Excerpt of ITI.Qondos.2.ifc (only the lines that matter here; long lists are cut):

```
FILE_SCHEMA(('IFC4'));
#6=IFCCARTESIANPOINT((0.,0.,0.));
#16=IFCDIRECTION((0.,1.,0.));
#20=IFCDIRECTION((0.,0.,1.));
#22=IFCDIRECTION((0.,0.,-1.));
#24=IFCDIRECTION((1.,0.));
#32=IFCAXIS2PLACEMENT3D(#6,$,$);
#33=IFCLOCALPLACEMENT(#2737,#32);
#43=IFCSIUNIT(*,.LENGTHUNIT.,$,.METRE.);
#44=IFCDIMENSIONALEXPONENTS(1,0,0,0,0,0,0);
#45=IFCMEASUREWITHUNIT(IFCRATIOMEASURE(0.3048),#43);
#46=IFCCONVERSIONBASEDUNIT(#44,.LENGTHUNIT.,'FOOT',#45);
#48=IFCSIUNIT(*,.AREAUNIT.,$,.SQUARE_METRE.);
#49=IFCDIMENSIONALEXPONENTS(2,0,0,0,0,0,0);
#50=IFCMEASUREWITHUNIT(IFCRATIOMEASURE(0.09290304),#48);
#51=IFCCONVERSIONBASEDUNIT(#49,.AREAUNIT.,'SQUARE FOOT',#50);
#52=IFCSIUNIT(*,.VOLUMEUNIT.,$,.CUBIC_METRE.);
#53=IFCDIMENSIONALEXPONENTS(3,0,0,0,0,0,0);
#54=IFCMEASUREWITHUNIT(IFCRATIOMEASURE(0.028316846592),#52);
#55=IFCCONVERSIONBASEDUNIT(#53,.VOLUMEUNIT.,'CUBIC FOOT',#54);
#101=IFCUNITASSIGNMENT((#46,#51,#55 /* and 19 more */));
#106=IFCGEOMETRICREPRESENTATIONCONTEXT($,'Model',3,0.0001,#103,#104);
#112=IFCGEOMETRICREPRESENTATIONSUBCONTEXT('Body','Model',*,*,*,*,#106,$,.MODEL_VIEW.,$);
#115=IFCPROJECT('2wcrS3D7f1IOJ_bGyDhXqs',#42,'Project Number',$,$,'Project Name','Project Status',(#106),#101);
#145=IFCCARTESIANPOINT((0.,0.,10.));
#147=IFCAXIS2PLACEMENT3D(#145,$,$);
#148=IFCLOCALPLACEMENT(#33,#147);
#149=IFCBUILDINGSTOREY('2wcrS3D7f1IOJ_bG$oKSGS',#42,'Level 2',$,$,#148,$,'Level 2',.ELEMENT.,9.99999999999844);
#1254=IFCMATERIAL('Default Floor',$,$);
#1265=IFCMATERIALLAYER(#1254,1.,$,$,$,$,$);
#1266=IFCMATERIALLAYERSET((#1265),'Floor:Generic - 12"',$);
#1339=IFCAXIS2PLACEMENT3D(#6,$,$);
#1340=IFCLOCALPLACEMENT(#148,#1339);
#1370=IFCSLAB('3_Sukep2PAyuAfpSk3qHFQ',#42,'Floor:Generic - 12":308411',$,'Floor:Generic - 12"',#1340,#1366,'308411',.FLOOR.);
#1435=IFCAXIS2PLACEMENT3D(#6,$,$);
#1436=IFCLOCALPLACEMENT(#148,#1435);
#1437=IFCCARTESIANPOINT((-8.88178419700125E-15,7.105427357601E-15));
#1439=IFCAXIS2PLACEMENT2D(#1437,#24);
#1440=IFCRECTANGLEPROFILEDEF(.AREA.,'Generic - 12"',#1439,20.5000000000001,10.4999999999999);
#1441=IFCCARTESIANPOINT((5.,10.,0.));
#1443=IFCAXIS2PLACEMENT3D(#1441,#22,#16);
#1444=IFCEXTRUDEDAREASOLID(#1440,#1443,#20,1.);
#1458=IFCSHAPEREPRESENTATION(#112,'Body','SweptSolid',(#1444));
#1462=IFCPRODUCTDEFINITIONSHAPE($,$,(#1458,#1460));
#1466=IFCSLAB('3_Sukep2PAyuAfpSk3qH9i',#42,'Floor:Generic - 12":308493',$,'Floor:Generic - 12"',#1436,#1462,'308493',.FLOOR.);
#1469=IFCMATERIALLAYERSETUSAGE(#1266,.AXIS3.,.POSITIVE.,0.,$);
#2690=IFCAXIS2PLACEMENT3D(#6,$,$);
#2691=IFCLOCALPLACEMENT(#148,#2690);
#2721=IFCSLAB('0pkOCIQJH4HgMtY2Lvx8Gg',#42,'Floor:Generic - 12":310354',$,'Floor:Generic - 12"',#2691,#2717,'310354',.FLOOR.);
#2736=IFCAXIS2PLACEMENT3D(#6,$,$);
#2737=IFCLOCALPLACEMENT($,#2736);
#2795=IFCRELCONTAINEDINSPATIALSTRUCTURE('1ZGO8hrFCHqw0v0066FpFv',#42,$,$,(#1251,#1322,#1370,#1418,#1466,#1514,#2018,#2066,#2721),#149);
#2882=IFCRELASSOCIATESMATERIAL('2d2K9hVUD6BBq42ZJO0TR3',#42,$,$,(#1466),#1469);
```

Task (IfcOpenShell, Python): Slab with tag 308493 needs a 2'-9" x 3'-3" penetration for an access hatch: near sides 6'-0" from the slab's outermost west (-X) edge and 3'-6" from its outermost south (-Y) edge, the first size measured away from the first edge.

```python
import numpy as np
import ifcopenshell
import ifcopenshell.api.feature
import ifcopenshell.api.geometry
import ifcopenshell.api.root
import ifcopenshell.geom
import ifcopenshell.util.placement
import ifcopenshell.util.representation
import ifcopenshell.util.shape
import ifcopenshell.util.unit

model = ifcopenshell.open("ITI.Qondos.2.ifc")
unit_scale = ifcopenshell.util.unit.calculate_unit_scale(model)
settings = ifcopenshell.geom.settings()


def volume(element):
    """Net volume in cubic metres, openings subtracted."""
    shape = ifcopenshell.geom.create_shape(settings, element)
    return ifcopenshell.util.shape.get_volume(shape.geometry)


slab = model.by_id(1466)
before = volume(slab)

# Extent in the slab's own axes, in metres. The edges named are its -X and -Y sides.
slab_shape = ifcopenshell.geom.create_shape(settings, slab)
vertices = ifcopenshell.util.shape.get_vertices(slab_shape.geometry)
x_min, y_min, bottom = vertices.min(axis=0)
top = vertices[:, 2].max()

opening = ifcopenshell.api.root.create_entity(model, ifc_class="IfcOpeningElement", name="Access hatch opening", predefined_type="OPENING")
context = ifcopenshell.util.representation.get_context(model, "Model", "Body", "MODEL_VIEW")
width, depth = 0.8382, 0.9906
outline = [(0.0, 0.0), (width, 0.0), (width, depth), (0.0, depth), (0.0, 0.0)]
# Overshoot both faces by 50 mm so the cut is clean.
shape = ifcopenshell.api.geometry.add_slab_representation(
    model, context=context, depth=top - bottom + 0.1, polyline=outline
)
ifcopenshell.api.geometry.assign_representation(model, product=opening, representation=shape)

matrix = ifcopenshell.util.placement.get_local_placement(slab.ObjectPlacement)
matrix[:, 3] = matrix @ np.append(np.array([x_min + 1.8288, y_min + 1.0668, bottom - 0.05]) / unit_scale, 1.0)
ifcopenshell.api.geometry.edit_object_placement(model, product=opening, matrix=matrix, is_si=False)
ifcopenshell.api.feature.add_feature(model, feature=opening, element=slab)

after = volume(slab)

print(f"slab volume {before:.3f} -> {after:.3f} m3")

model.write("ITI.Qondos.2_edited.ifc")
```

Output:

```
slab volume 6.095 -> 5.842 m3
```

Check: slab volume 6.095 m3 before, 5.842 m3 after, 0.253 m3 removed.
